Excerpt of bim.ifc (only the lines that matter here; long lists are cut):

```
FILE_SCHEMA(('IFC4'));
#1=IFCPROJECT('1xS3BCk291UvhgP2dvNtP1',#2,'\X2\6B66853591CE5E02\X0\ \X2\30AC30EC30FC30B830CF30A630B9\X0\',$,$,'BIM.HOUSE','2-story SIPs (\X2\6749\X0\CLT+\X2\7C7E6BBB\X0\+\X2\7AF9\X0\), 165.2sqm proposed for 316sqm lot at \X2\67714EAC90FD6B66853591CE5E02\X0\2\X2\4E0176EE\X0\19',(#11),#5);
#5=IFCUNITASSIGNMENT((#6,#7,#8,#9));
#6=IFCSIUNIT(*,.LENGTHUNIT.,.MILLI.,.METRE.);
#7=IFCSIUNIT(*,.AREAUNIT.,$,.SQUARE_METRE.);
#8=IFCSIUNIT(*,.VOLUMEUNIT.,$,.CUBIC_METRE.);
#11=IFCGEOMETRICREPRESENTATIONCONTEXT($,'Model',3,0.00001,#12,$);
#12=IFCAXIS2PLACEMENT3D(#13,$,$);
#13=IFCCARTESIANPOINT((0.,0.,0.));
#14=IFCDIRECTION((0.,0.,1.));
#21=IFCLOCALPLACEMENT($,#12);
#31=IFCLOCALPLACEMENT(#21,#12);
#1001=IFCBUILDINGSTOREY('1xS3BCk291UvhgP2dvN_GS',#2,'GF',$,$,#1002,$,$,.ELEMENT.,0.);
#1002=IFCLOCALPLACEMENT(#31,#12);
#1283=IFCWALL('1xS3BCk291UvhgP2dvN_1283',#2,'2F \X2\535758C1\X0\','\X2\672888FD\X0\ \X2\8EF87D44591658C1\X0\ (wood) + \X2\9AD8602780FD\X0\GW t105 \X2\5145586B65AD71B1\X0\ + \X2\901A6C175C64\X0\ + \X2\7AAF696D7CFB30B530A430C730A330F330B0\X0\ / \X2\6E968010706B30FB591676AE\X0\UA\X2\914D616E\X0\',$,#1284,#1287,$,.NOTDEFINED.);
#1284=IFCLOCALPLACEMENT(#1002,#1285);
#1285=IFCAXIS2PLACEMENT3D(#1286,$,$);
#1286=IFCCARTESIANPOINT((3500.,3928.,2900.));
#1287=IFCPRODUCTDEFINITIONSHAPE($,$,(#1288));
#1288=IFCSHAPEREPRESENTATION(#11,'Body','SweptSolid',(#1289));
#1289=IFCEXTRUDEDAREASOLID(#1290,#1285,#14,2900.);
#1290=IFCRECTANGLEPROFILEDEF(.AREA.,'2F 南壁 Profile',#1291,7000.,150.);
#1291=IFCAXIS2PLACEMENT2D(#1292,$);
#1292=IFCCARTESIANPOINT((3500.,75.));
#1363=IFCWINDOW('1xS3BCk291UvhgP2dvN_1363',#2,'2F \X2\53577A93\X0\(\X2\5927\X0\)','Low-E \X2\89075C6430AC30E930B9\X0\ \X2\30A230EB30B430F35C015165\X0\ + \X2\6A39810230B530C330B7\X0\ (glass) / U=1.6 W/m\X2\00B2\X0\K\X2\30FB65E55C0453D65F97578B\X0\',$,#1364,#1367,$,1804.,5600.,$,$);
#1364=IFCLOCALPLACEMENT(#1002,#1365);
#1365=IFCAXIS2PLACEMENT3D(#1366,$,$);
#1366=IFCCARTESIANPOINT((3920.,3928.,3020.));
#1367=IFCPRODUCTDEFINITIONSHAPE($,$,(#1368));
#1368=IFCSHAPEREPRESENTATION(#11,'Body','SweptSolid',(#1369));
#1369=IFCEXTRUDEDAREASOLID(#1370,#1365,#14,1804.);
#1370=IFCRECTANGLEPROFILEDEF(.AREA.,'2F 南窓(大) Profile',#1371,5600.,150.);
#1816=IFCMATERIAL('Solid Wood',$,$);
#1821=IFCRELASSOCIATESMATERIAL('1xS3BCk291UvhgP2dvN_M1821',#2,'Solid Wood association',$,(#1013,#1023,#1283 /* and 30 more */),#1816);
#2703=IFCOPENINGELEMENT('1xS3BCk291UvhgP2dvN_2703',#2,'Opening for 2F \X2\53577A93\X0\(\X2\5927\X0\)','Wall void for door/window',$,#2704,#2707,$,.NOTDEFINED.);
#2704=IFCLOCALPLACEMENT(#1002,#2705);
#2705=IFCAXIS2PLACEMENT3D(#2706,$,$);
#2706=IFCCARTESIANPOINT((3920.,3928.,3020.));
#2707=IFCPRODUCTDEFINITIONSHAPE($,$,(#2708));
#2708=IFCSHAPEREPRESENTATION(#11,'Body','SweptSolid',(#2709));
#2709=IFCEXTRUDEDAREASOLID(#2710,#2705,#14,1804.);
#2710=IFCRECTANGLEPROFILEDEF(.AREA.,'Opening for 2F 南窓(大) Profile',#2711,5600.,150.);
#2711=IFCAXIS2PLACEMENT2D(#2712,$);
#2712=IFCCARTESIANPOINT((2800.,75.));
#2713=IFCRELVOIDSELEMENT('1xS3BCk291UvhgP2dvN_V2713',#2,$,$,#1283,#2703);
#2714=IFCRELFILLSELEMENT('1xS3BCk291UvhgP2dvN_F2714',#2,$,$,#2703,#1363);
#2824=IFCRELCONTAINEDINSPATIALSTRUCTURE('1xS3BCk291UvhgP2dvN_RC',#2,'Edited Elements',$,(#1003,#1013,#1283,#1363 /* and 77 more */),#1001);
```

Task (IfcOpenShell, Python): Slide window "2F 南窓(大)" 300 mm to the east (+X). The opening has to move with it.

```python
import ifcopenshell
import ifcopenshell.api.geometry
import ifcopenshell.util.placement

model = ifcopenshell.open("bim.ifc")

window = model.by_id(1363)
opening = window.FillsVoids[0].RelatingOpeningElement
wall = opening.VoidsElements[0].RelatingBuildingElement

wall_matrix = ifcopenshell.util.placement.get_local_placement(wall.ObjectPlacement)
shift = wall_matrix[:3, 0] * 300.0
before = ifcopenshell.util.placement.get_local_placement(window.ObjectPlacement)[:3, 3].copy()

# The window is not placed relative to its opening, so move both.
for product in (opening, window):
    matrix = ifcopenshell.util.placement.get_local_placement(product.ObjectPlacement)
    matrix[:3, 3] += shift
    ifcopenshell.api.geometry.edit_object_placement(model, product=product, matrix=matrix, is_si=False)

after = ifcopenshell.util.placement.get_local_placement(window.ObjectPlacement)[:3, 3]
print("window moved by", (after - before).round(3) + 0.0)

model.write("bim_updated.ifc")
```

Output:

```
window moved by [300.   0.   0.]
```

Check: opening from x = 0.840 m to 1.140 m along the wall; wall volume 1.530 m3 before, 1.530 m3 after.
